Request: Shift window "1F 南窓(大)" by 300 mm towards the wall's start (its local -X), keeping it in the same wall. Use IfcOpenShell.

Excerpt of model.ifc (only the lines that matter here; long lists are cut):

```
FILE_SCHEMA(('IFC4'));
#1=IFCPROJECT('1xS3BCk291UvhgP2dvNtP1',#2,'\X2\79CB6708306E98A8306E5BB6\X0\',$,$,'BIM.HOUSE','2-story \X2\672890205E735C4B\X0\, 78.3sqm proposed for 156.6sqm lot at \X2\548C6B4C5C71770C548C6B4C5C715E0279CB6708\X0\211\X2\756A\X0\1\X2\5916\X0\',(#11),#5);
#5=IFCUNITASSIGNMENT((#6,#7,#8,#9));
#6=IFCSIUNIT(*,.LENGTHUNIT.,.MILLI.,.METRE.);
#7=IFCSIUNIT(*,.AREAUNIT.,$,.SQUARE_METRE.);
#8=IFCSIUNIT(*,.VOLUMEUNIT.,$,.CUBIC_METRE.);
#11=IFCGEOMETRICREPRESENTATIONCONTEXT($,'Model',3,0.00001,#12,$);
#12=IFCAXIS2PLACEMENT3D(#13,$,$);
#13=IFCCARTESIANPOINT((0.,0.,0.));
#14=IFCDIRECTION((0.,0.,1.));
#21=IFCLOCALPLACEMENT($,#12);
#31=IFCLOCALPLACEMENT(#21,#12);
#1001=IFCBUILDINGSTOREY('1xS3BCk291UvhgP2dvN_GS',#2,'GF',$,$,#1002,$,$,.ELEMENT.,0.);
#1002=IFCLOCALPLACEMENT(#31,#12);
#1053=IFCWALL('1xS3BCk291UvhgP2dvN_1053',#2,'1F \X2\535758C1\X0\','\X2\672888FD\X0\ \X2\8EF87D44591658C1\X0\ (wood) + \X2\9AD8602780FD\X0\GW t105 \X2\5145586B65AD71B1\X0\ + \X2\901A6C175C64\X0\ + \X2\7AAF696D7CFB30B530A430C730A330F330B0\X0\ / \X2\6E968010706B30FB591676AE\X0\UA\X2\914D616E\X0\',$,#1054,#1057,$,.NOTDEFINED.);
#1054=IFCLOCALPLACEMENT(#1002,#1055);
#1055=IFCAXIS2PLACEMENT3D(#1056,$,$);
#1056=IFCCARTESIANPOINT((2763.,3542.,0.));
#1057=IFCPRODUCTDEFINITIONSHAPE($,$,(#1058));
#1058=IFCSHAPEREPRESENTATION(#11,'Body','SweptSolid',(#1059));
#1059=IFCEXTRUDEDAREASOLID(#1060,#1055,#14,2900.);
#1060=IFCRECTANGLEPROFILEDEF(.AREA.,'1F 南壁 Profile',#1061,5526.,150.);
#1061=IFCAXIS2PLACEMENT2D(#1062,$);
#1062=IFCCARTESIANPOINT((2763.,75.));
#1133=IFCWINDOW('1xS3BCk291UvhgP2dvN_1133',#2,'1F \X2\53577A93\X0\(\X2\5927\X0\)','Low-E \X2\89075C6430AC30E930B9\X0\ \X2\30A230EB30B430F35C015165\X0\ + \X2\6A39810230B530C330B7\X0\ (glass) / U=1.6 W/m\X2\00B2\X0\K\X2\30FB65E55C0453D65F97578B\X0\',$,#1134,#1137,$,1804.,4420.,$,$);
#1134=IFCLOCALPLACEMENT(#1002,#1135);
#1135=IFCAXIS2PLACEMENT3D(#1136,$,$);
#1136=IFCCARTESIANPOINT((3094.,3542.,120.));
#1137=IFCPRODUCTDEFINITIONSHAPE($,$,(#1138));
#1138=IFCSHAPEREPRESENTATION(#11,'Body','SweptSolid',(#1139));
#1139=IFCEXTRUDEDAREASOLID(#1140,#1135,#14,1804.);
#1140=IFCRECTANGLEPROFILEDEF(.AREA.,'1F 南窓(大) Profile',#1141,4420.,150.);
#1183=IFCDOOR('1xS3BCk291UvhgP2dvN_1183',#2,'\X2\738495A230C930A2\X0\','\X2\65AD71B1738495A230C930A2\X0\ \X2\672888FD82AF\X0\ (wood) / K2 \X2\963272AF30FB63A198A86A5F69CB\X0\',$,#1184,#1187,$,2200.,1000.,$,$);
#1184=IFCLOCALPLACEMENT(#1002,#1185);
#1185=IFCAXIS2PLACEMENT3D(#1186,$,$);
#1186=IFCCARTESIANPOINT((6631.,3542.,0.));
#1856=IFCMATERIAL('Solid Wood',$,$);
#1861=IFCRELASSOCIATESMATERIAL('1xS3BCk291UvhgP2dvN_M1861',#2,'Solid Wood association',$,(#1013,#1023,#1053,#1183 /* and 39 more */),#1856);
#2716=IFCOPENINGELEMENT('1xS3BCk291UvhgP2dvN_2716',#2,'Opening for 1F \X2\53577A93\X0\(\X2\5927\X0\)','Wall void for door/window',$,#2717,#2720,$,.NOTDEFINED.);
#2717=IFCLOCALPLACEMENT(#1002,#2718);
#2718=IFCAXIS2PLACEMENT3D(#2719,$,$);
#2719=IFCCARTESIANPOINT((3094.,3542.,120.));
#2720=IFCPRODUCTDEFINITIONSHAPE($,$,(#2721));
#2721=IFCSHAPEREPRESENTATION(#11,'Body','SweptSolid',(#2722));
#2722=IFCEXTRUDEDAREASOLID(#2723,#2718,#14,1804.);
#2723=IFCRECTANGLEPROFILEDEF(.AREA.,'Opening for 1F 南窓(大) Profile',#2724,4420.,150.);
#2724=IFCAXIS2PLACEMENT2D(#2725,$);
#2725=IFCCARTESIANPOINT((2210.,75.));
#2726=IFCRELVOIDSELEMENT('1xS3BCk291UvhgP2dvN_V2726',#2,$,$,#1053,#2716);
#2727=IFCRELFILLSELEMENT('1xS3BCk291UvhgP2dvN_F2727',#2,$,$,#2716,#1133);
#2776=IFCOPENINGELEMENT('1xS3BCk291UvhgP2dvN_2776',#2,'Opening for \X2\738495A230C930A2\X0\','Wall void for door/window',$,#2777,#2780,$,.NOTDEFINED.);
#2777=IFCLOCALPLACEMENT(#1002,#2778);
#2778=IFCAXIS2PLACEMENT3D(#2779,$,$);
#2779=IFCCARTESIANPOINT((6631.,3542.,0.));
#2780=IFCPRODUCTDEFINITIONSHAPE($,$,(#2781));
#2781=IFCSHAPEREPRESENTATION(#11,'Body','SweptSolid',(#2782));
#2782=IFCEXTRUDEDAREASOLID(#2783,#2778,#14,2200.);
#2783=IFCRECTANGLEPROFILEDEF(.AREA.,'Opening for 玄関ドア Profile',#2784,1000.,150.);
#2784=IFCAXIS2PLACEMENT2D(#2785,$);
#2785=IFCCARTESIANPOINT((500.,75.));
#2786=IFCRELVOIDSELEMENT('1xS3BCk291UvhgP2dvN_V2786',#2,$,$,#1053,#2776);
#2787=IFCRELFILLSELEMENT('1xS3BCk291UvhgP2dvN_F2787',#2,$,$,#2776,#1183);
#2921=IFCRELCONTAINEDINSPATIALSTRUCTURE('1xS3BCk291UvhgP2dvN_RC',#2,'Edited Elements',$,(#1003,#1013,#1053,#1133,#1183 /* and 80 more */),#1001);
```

```python
import ifcopenshell
import ifcopenshell.api.geometry
import ifcopenshell.util.placement
import ifcopenshell.util.unit

model = ifcopenshell.open("model.ifc")
unit_scale = ifcopenshell.util.unit.calculate_unit_scale(model)

window = model.by_guid("1xS3BCk291UvhgP2dvN_1133")
opening = window.FillsVoids[0].RelatingOpeningElement
wall = opening.VoidsElements[0].RelatingBuildingElement

wall_matrix = ifcopenshell.util.placement.get_local_placement(wall.ObjectPlacement)
shift = wall_matrix[:3, 0] * -0.3 / unit_scale
before = ifcopenshell.util.placement.get_local_placement(window.ObjectPlacement)[:3, 3].copy()

# The window is not placed relative to its opening, so move both.
for product in (opening, window):
    matrix = ifcopenshell.util.placement.get_local_placement(product.ObjectPlacement)
    matrix[:3, 3] += shift
    ifcopenshell.api.geometry.edit_object_placement(model, product=product, matrix=matrix, is_si=False)

after = ifcopenshell.util.placement.get_local_placement(window.ObjectPlacement)[:3, 3]
print("window moved by", (after - before).round(3) + 0.0)

model.write("model_v2.ifc")
```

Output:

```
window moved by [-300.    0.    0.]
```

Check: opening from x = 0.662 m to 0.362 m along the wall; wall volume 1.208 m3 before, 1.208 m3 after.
